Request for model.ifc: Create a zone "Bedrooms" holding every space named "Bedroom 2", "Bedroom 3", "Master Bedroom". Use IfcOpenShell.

First a look at what the model holds.

```python
import ifcopenshell

model = ifcopenshell.open("model.ifc")
print(model.schema)
seen = {}
for space in model.by_type("IfcSpace"):
    seen[space.Name] = seen.get(space.Name, 0) + 1
for name, count in sorted(seen.items(), key=str):
    print(count, "x", name)
print("zones:", [z.Name for z in model.by_type("IfcZone")][:20])
```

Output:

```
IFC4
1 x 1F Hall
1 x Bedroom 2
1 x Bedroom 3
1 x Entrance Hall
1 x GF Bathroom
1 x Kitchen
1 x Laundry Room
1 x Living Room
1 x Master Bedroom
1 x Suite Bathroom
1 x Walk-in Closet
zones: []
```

```python
import ifcopenshell
import ifcopenshell.api.group
import ifcopenshell.api.root

model = ifcopenshell.open("model.ifc")

names = {"Bedroom 2", "Bedroom 3", "Master Bedroom"}
spaces = [s for s in model.by_type("IfcSpace") if s.Name in names]

zone = ifcopenshell.api.root.create_entity(model, ifc_class="IfcZone", name="Bedrooms")
ifcopenshell.api.group.assign_group(model, products=spaces, group=zone)
print(len(spaces), "spaces in", zone.Name)

model.write("model-out.ifc")
```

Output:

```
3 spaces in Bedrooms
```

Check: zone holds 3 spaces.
